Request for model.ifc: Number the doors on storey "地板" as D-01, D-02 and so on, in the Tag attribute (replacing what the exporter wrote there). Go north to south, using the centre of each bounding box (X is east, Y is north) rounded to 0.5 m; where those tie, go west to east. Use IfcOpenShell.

First a look at what the model holds.

```python
import ifcopenshell
import ifcopenshell.util.element
import ifcopenshell.util.placement

model = ifcopenshell.open("model.ifc")
print(model.schema)
storey = next(s for s in model.by_type("IfcBuildingStorey") if s.Name == "地板")
doors = [e for e in ifcopenshell.util.element.get_decomposition(storey) if e.is_a("IfcDoor")]
for e in sorted(doors, key=lambda e: e.id()):
    origin = ifcopenshell.util.placement.get_local_placement(e.ObjectPlacement)[:3, 3]
    print(e.id(), e.Tag, e.Name, origin.round(2) + 0.0, sep=" | ")
```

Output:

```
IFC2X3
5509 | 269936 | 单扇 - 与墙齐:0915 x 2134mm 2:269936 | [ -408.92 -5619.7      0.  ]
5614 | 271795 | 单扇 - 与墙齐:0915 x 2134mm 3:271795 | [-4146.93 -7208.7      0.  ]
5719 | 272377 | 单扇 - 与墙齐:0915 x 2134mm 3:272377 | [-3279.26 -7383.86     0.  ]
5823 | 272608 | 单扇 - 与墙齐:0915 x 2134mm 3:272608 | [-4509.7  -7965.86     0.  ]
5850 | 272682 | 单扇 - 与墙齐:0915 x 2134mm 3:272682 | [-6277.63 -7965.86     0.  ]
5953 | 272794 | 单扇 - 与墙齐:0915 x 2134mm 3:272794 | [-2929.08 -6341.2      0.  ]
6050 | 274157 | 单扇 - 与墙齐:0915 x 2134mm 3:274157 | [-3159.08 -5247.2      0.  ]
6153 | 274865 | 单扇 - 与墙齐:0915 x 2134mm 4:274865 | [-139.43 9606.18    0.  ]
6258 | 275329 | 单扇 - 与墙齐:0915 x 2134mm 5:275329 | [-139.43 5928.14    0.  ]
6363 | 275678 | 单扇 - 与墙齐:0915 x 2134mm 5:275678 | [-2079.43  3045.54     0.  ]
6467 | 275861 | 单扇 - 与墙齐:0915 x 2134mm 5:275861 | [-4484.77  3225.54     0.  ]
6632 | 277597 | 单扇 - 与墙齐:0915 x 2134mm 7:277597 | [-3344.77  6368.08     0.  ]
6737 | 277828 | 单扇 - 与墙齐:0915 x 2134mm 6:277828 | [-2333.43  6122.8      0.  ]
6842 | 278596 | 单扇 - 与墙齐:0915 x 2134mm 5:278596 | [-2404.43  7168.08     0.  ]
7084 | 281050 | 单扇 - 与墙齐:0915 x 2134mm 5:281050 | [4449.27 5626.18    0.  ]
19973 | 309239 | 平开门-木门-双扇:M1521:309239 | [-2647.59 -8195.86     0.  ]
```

```python
import ifcopenshell
import ifcopenshell.geom
import ifcopenshell.util.element
import ifcopenshell.util.shape

model = ifcopenshell.open("model.ifc")
settings = ifcopenshell.geom.settings()
settings.set("use-world-coords", True)


def centre(element):
    shape = ifcopenshell.geom.create_shape(settings, element)
    return ifcopenshell.util.shape.get_bbox_centroid(shape.geometry)


storey = next(s for s in model.by_type("IfcBuildingStorey") if s.Name == "地板")
doors = [e for e in ifcopenshell.util.element.get_decomposition(storey) if e.is_a("IfcDoor")]

# Insertion points can sit at a corner or the storey origin, so sort by the geometry (in metres).
centres = {e: centre(e) for e in doors}
doors.sort(key=lambda e: (-round(centres[e][1] / 0.5), centres[e][0]))

for i, e in enumerate(doors, start=1):
    number = f"D-{i:02d}"
    e.Tag = number
    print(e.id(), number)

model.write("model_edited.ifc")
```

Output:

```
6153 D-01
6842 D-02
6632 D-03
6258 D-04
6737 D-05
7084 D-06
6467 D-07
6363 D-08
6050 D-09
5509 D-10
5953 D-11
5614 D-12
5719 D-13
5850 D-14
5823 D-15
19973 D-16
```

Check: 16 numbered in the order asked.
